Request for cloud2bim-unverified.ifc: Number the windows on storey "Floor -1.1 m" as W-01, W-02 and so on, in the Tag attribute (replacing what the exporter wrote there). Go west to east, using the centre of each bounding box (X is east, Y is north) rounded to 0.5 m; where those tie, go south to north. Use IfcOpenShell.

First a look at what the model holds.

```python
import ifcopenshell
import ifcopenshell.util.element
import ifcopenshell.util.placement

model = ifcopenshell.open("cloud2bim-unverified.ifc")
print(model.schema)
storey = next(s for s in model.by_type("IfcBuildingStorey") if s.Name == "Floor -1.1 m")
windows = [e for e in ifcopenshell.util.element.get_decomposition(storey) if e.is_a("IfcWindow")]
for e in sorted(windows, key=lambda e: e.id()):
    origin = ifcopenshell.util.placement.get_local_placement(e.ObjectPlacement)[:3, 3]
    print(e.id(), e.Tag, e.Name, origin.round(2) + 0.0, sep=" | ")
```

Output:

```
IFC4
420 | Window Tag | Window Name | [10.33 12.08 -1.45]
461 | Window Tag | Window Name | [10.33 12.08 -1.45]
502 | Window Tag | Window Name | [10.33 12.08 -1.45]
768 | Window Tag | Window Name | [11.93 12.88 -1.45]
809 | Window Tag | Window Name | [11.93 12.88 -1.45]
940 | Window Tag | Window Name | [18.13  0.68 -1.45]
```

```python
import ifcopenshell
import ifcopenshell.geom
import ifcopenshell.util.element
import ifcopenshell.util.shape

model = ifcopenshell.open("cloud2bim-unverified.ifc")
settings = ifcopenshell.geom.settings()
settings.set("use-world-coords", True)


def centre(element):
    shape = ifcopenshell.geom.create_shape(settings, element)
    return ifcopenshell.util.shape.get_bbox_centroid(shape.geometry)


storey = next(s for s in model.by_type("IfcBuildingStorey") if s.Name == "Floor -1.1 m")
windows = [e for e in ifcopenshell.util.element.get_decomposition(storey) if e.is_a("IfcWindow")]

# Insertion points can sit at a corner or the storey origin, so sort by the geometry (in metres).
centres = {e: centre(e) for e in windows}
windows.sort(key=lambda e: (round(centres[e][0] / 0.5), centres[e][1]))

for i, e in enumerate(windows, start=1):
    number = f"W-{i:02d}"
    e.Tag = number
    print(e.id(), number)

model.write("cloud2bim-unverified_edited.ifc")
```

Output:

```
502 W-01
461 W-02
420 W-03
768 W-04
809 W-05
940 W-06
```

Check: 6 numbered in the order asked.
